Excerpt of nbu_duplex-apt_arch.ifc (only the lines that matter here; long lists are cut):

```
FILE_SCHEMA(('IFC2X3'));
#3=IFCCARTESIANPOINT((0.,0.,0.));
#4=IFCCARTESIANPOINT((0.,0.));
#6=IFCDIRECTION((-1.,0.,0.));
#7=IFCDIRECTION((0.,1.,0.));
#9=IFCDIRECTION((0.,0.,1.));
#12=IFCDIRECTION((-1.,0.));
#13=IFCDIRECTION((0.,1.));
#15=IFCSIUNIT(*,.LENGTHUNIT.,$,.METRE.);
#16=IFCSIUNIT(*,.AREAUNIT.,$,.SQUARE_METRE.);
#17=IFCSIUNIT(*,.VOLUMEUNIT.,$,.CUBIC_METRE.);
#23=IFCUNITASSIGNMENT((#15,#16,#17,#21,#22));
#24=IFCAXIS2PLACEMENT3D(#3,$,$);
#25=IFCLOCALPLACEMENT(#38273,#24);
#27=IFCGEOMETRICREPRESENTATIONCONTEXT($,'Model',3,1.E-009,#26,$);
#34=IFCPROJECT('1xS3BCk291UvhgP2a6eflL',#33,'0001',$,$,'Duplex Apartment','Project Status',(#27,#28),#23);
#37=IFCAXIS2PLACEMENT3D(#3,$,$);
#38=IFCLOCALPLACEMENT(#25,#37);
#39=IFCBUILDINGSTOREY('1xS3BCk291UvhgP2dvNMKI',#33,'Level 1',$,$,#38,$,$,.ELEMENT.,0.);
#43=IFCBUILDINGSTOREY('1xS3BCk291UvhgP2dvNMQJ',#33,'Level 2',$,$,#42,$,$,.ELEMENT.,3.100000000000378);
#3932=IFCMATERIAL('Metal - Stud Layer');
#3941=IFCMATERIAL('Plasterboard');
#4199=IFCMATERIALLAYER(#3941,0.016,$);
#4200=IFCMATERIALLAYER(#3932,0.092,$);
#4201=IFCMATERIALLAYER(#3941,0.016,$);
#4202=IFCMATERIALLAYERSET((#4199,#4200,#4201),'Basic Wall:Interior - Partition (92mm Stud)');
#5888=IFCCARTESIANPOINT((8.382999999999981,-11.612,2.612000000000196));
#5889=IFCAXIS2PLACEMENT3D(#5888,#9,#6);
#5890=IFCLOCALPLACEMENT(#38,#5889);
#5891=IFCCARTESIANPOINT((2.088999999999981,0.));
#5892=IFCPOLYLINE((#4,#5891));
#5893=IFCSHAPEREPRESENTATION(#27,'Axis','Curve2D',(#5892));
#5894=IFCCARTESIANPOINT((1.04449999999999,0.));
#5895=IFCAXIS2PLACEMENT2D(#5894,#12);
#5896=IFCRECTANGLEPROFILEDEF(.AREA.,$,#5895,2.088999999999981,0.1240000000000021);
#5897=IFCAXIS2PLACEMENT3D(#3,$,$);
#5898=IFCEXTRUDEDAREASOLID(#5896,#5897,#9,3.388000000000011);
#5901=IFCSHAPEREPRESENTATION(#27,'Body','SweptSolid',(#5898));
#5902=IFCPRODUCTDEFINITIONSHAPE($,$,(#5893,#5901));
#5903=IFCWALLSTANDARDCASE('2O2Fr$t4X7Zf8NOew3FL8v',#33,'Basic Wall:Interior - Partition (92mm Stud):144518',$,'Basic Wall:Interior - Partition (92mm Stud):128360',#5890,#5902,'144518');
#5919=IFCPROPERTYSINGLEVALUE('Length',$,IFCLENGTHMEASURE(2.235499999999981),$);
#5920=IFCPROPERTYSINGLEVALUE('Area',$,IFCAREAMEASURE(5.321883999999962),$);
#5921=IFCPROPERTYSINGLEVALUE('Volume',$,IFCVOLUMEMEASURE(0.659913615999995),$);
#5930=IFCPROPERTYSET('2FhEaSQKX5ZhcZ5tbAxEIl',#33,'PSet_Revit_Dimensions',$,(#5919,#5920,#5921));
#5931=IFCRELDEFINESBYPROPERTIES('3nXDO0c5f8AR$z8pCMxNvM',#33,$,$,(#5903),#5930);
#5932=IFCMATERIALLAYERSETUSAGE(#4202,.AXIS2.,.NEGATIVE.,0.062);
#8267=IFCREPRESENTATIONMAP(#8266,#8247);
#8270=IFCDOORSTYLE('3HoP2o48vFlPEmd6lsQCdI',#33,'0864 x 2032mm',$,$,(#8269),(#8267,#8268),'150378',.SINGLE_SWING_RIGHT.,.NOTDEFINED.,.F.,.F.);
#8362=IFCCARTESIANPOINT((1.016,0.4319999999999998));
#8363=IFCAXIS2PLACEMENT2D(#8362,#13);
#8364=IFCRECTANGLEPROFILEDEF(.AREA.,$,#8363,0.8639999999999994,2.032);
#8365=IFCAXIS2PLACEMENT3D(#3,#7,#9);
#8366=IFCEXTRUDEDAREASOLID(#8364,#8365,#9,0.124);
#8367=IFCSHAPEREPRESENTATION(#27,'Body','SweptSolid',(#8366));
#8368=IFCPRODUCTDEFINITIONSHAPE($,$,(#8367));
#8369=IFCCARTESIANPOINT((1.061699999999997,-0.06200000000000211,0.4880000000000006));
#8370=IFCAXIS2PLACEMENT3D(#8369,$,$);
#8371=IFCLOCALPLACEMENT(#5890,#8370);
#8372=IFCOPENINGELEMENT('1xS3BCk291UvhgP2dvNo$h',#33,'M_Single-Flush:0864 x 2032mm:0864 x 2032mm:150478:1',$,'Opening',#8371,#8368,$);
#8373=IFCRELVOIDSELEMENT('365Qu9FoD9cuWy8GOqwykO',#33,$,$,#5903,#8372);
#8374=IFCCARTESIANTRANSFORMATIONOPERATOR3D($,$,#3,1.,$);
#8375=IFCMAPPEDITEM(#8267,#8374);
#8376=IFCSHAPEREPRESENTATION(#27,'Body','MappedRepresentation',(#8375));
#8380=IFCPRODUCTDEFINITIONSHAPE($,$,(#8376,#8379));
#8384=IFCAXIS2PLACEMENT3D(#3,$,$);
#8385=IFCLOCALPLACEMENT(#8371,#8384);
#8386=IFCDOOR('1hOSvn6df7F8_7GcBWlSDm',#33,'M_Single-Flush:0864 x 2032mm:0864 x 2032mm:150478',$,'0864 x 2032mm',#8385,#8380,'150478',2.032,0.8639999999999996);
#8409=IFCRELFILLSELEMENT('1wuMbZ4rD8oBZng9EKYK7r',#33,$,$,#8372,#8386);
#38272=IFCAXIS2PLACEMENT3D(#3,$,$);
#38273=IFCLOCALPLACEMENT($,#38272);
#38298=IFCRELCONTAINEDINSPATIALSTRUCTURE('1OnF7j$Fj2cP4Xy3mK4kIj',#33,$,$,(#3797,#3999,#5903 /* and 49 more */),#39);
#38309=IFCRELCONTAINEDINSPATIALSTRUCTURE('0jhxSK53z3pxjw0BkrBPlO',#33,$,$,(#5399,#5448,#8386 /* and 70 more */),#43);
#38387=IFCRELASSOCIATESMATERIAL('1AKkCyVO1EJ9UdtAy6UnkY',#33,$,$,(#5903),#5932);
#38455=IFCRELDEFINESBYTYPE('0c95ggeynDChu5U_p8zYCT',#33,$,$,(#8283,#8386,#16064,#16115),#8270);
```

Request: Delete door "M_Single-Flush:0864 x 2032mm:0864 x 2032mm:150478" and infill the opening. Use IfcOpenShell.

```python
import ifcopenshell
import ifcopenshell.api.feature
import ifcopenshell.api.pset
import ifcopenshell.api.root
import ifcopenshell.geom
import ifcopenshell.util.element
import ifcopenshell.util.shape
import ifcopenshell.util.unit

model = ifcopenshell.open("nbu_duplex-apt_arch.ifc")
area_scale = ifcopenshell.util.unit.calculate_unit_scale(model, "AREAUNIT")
volume_scale = ifcopenshell.util.unit.calculate_unit_scale(model, "VOLUMEUNIT")
settings = ifcopenshell.geom.settings()


def volume(element):
    """Net volume in cubic metres, openings subtracted."""
    shape = ifcopenshell.geom.create_shape(settings, element)
    return ifcopenshell.util.shape.get_volume(shape.geometry)


door = model.by_guid("1hOSvn6df7F8_7GcBWlSDm")
opening = door.FillsVoids[0].RelatingOpeningElement
wall = opening.VoidsElements[0].RelatingBuildingElement
before = volume(wall)

ifcopenshell.api.root.remove_product(model, product=door)
ifcopenshell.api.feature.remove_feature(model, feature=opening)

after = volume(wall)
thickness = 0.124  # wall thickness in metres

# Update the wall's stored quantities.
pset = model.by_id(ifcopenshell.util.element.get_pset(wall, "PSet_Revit_Dimensions", should_inherit=False)["id"])
ifcopenshell.api.pset.edit_pset(model, pset=pset, properties={
    "Area": model.create_entity("IfcAreaMeasure", after / thickness / area_scale),
    "Volume": model.create_entity("IfcVolumeMeasure", after / volume_scale),
})

print(f"wall volume {before:.3f} -> {after:.3f} m3")

model.write("nbu_duplex-apt_arch_updated.ifc")
```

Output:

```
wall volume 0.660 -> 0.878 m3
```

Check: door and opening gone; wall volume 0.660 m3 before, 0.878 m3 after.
